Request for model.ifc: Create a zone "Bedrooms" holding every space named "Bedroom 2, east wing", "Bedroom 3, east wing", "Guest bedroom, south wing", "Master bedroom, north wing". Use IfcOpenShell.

First a look at what the model holds.

```python
import ifcopenshell

model = ifcopenshell.open("model.ifc")
print(model.schema)
seen = {}
for space in model.by_type("IfcSpace"):
    seen[space.LongName] = seen.get(space.LongName, 0) + 1
for name, count in sorted(seen.items(), key=str):
    print(count, "x", name)
print("zones:", [z.Name for z in model.by_type("IfcZone")][:20])
```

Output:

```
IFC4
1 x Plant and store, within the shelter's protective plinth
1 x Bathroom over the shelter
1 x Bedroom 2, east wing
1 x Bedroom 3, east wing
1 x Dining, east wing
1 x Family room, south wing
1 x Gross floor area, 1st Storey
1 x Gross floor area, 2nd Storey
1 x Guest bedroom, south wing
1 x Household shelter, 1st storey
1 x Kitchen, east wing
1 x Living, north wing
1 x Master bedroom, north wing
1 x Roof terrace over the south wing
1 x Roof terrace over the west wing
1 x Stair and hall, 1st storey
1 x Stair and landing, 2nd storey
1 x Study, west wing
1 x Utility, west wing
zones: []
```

```python
import ifcopenshell
import ifcopenshell.api.group
import ifcopenshell.api.root

model = ifcopenshell.open("model.ifc")

names = {"Bedroom 2, east wing", "Bedroom 3, east wing", "Guest bedroom, south wing", "Master bedroom, north wing"}
spaces = [s for s in model.by_type("IfcSpace") if s.LongName in names]

zone = ifcopenshell.api.root.create_entity(model, ifc_class="IfcZone", name="Bedrooms")
ifcopenshell.api.group.assign_group(model, products=spaces, group=zone)
print(len(spaces), "spaces in", zone.Name)

model.write("model_v2.ifc")
```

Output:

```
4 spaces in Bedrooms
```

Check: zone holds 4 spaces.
